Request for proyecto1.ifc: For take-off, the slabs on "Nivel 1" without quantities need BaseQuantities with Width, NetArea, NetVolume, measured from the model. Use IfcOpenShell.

First a look at what the model holds.

```python
import ifcopenshell
import ifcopenshell.util.element
import ifcopenshell.util.unit

model = ifcopenshell.open("proyecto1.ifc")
print(model.schema)
for unit_type in ("LENGTHUNIT", "AREAUNIT", "VOLUMEUNIT"):
    print(unit_type, ifcopenshell.util.unit.calculate_unit_scale(model, unit_type))
storey = next(s for s in model.by_type("IfcBuildingStorey") if s.Name == "Nivel 1")
slabs = [e for e in ifcopenshell.util.element.get_decomposition(storey) if e.is_a("IfcSlab")]
for e in sorted(slabs, key=lambda e: e.id()):
    print(e.id(), e.is_a(), e.Name, list(ifcopenshell.util.element.get_psets(e, qtos_only=True)), sep=" | ")
```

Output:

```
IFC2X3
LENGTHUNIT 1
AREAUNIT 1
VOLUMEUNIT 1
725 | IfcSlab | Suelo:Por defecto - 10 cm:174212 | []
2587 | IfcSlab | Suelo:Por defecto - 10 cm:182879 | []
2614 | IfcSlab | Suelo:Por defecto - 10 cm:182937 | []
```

```python
import ifcopenshell
import ifcopenshell.api.pset
import ifcopenshell.geom
import ifcopenshell.util.element
import ifcopenshell.util.shape
import ifcopenshell.util.unit

model = ifcopenshell.open("proyecto1.ifc")
unit_scale = ifcopenshell.util.unit.calculate_unit_scale(model)
area_scale = ifcopenshell.util.unit.calculate_unit_scale(model, "AREAUNIT")
volume_scale = ifcopenshell.util.unit.calculate_unit_scale(model, "VOLUMEUNIT")
settings = ifcopenshell.geom.settings()

storey = next(s for s in model.by_type("IfcBuildingStorey") if s.Name == "Nivel 1")
slabs = [e for e in ifcopenshell.util.element.get_decomposition(storey) if e.is_a("IfcSlab")]

for e in sorted(slabs, key=lambda e: e.id()):
    if ifcopenshell.util.element.get_psets(e, qtos_only=True, should_inherit=False):
        continue
    # Geometry comes back in metres, in the element's own axes.
    shape = ifcopenshell.geom.create_shape(settings, e)
    values = {
        "Width": ifcopenshell.util.shape.get_z(shape.geometry) / unit_scale,
        "NetArea": ifcopenshell.util.shape.get_footprint_area(shape.geometry) / area_scale,
        "NetVolume": ifcopenshell.util.shape.get_volume(shape.geometry) / volume_scale,
    }
    qto = ifcopenshell.api.pset.add_qto(model, product=e, name="BaseQuantities")
    ifcopenshell.api.pset.edit_qto(model, qto=qto, properties=values)
    print(e.id(), {k: round(v, 3) for k, v in values.items()})

model.write("proyecto1_edited.ifc")
```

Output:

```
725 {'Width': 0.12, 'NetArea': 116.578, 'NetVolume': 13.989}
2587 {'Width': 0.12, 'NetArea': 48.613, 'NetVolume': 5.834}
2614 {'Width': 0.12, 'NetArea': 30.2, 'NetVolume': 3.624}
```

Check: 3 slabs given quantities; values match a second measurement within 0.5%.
